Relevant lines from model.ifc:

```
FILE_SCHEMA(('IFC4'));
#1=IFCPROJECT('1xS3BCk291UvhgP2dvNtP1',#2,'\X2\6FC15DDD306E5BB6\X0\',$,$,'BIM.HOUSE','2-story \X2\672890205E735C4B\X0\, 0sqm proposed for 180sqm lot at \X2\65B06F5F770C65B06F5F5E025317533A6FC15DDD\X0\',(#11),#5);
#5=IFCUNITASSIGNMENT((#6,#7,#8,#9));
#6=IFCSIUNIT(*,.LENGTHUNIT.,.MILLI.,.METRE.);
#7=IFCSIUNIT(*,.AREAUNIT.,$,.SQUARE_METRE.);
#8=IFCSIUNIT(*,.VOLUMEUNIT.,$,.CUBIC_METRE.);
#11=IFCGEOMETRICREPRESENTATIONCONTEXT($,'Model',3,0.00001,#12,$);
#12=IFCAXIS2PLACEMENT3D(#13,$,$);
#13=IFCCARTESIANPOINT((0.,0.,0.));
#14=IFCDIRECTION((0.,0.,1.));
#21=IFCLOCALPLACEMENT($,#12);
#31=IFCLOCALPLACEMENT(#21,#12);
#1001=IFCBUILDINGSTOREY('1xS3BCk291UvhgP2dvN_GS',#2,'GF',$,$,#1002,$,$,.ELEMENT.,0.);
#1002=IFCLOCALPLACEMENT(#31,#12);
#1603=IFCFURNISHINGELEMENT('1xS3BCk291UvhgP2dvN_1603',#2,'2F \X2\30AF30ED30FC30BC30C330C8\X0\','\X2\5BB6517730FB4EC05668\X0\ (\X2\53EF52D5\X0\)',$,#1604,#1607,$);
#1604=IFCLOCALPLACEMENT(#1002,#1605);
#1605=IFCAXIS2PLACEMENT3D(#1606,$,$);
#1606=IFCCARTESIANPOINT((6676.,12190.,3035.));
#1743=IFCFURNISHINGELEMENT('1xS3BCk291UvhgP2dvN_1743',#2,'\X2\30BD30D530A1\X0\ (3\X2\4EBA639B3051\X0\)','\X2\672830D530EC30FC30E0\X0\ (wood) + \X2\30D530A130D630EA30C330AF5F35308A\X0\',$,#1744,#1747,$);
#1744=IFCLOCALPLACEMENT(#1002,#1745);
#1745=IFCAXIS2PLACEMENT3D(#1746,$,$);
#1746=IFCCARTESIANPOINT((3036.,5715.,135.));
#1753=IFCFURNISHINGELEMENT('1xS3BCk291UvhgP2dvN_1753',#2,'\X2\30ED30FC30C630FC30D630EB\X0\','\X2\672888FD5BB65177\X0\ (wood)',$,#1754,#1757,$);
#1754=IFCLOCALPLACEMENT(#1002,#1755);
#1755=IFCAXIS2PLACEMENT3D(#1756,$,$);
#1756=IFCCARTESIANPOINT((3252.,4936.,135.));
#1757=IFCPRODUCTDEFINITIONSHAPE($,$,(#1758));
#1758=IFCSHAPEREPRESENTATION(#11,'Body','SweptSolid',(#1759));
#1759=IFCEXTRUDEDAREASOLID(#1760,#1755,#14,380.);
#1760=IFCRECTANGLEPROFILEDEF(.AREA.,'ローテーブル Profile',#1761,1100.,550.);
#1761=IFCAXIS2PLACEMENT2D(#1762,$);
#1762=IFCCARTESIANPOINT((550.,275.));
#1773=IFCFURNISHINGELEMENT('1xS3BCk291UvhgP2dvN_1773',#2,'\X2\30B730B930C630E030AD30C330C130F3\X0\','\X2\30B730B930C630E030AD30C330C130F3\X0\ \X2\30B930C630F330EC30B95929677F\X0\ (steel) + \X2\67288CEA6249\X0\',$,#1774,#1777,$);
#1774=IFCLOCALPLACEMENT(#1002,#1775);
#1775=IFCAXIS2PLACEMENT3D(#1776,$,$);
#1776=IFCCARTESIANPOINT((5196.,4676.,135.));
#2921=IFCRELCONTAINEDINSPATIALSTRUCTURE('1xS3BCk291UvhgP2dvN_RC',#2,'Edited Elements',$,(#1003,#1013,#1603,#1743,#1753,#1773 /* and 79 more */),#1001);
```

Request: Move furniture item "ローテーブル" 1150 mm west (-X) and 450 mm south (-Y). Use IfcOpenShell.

```python
import ifcopenshell
import ifcopenshell.api.geometry
import ifcopenshell.util.placement

model = ifcopenshell.open("model.ifc")

item = model.by_id(1753)
matrix = ifcopenshell.util.placement.get_local_placement(item.ObjectPlacement)
matrix[0, 3] -= 1150.0
matrix[1, 3] -= 450.0
ifcopenshell.api.geometry.edit_object_placement(model, product=item, matrix=matrix, is_si=False)

print(ifcopenshell.util.placement.get_local_placement(item.ObjectPlacement).round(3) + 0.0)

model.write("model_updated.ifc")
```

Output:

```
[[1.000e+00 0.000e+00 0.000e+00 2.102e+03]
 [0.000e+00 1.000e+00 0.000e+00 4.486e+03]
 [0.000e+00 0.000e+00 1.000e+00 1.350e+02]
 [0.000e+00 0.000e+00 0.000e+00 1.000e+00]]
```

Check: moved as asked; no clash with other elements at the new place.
